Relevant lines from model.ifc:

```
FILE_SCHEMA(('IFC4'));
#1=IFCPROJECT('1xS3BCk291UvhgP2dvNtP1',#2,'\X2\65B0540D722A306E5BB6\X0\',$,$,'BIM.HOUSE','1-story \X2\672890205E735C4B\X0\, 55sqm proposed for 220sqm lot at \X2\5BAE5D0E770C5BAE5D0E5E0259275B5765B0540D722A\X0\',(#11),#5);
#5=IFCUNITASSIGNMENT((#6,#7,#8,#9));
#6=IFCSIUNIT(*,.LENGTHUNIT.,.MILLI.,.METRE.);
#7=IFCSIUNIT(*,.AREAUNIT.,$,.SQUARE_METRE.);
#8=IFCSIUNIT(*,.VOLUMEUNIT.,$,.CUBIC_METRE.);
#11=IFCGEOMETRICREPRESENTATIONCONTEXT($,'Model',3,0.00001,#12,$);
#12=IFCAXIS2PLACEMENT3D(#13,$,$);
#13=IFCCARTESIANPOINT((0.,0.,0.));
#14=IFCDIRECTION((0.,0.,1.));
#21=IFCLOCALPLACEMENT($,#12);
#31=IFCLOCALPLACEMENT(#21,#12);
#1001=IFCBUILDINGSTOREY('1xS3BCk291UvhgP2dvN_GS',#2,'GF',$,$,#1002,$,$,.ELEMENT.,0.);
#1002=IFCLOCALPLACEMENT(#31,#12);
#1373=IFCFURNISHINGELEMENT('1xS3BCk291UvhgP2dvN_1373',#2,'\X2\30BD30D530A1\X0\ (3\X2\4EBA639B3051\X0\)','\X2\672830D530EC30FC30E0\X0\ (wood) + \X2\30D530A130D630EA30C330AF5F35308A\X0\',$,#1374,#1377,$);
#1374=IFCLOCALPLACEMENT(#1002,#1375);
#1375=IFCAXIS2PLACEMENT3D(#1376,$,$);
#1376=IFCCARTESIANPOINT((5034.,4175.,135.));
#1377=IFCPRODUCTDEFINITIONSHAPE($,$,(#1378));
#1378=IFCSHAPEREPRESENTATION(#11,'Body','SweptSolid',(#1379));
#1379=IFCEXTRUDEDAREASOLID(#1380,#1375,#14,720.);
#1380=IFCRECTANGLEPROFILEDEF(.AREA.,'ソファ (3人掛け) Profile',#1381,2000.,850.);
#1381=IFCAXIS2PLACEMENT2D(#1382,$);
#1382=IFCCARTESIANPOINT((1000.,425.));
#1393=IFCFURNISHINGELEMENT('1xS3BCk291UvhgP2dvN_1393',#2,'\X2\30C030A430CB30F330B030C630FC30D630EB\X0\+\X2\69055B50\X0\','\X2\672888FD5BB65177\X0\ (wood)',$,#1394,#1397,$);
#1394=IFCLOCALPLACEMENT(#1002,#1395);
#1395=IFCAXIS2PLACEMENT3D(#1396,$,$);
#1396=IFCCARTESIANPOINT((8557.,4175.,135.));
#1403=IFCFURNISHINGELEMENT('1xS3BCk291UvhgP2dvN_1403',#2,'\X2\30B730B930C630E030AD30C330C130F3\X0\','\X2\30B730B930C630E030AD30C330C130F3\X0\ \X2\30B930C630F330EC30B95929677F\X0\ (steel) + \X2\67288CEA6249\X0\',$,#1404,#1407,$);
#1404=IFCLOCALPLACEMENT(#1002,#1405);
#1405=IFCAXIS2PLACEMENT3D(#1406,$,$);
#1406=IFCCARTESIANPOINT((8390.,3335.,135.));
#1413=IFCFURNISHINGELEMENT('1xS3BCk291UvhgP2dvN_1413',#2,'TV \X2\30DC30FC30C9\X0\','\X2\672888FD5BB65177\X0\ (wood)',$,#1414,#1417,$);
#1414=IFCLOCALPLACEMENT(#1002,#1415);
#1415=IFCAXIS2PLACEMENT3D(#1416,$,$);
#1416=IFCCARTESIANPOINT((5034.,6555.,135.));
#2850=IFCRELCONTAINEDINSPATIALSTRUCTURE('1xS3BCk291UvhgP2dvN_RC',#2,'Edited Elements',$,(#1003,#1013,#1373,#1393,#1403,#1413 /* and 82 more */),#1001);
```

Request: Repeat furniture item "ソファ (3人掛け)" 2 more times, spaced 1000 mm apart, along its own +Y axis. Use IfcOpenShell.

```python
import ifcopenshell
import ifcopenshell.api.geometry
import ifcopenshell.api.root
import ifcopenshell.util.element
import ifcopenshell.util.placement

model = ifcopenshell.open("model.ifc")


def reuse_history(source, copy):
    """copy_class also copies each property set's owner history, people and application; keep the originals."""
    for rel in copy.IsDefinedBy:
        if rel.is_a("IfcRelDefinesByProperties") and (history := rel.RelatingPropertyDefinition.OwnerHistory):
            rel.RelatingPropertyDefinition.OwnerHistory = source.OwnerHistory
            ifcopenshell.util.element.remove_deep2(model, history)


source = model.by_guid("1xS3BCk291UvhgP2dvN_1373")
base = ifcopenshell.util.placement.get_local_placement(source.ObjectPlacement)
step = base[:3, 1] * 1000.0

for i in range(1, 3):
    copy = ifcopenshell.api.root.copy_class(model, product=source)
    copy.Representation = ifcopenshell.util.element.copy_deep(
        model, source.Representation, exclude=["IfcGeometricRepresentationContext", "IfcRepresentationMap"]
    )
    reuse_history(source, copy)
    matrix = base.copy()
    matrix[:3, 3] += i * step
    print("added at", matrix[:3, 3].round(3) + 0.0)
    ifcopenshell.api.geometry.edit_object_placement(model, product=copy, matrix=matrix, is_si=False)

model.write("model_rev.ifc")
```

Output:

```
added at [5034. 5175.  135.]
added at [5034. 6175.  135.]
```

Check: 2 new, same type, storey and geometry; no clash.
